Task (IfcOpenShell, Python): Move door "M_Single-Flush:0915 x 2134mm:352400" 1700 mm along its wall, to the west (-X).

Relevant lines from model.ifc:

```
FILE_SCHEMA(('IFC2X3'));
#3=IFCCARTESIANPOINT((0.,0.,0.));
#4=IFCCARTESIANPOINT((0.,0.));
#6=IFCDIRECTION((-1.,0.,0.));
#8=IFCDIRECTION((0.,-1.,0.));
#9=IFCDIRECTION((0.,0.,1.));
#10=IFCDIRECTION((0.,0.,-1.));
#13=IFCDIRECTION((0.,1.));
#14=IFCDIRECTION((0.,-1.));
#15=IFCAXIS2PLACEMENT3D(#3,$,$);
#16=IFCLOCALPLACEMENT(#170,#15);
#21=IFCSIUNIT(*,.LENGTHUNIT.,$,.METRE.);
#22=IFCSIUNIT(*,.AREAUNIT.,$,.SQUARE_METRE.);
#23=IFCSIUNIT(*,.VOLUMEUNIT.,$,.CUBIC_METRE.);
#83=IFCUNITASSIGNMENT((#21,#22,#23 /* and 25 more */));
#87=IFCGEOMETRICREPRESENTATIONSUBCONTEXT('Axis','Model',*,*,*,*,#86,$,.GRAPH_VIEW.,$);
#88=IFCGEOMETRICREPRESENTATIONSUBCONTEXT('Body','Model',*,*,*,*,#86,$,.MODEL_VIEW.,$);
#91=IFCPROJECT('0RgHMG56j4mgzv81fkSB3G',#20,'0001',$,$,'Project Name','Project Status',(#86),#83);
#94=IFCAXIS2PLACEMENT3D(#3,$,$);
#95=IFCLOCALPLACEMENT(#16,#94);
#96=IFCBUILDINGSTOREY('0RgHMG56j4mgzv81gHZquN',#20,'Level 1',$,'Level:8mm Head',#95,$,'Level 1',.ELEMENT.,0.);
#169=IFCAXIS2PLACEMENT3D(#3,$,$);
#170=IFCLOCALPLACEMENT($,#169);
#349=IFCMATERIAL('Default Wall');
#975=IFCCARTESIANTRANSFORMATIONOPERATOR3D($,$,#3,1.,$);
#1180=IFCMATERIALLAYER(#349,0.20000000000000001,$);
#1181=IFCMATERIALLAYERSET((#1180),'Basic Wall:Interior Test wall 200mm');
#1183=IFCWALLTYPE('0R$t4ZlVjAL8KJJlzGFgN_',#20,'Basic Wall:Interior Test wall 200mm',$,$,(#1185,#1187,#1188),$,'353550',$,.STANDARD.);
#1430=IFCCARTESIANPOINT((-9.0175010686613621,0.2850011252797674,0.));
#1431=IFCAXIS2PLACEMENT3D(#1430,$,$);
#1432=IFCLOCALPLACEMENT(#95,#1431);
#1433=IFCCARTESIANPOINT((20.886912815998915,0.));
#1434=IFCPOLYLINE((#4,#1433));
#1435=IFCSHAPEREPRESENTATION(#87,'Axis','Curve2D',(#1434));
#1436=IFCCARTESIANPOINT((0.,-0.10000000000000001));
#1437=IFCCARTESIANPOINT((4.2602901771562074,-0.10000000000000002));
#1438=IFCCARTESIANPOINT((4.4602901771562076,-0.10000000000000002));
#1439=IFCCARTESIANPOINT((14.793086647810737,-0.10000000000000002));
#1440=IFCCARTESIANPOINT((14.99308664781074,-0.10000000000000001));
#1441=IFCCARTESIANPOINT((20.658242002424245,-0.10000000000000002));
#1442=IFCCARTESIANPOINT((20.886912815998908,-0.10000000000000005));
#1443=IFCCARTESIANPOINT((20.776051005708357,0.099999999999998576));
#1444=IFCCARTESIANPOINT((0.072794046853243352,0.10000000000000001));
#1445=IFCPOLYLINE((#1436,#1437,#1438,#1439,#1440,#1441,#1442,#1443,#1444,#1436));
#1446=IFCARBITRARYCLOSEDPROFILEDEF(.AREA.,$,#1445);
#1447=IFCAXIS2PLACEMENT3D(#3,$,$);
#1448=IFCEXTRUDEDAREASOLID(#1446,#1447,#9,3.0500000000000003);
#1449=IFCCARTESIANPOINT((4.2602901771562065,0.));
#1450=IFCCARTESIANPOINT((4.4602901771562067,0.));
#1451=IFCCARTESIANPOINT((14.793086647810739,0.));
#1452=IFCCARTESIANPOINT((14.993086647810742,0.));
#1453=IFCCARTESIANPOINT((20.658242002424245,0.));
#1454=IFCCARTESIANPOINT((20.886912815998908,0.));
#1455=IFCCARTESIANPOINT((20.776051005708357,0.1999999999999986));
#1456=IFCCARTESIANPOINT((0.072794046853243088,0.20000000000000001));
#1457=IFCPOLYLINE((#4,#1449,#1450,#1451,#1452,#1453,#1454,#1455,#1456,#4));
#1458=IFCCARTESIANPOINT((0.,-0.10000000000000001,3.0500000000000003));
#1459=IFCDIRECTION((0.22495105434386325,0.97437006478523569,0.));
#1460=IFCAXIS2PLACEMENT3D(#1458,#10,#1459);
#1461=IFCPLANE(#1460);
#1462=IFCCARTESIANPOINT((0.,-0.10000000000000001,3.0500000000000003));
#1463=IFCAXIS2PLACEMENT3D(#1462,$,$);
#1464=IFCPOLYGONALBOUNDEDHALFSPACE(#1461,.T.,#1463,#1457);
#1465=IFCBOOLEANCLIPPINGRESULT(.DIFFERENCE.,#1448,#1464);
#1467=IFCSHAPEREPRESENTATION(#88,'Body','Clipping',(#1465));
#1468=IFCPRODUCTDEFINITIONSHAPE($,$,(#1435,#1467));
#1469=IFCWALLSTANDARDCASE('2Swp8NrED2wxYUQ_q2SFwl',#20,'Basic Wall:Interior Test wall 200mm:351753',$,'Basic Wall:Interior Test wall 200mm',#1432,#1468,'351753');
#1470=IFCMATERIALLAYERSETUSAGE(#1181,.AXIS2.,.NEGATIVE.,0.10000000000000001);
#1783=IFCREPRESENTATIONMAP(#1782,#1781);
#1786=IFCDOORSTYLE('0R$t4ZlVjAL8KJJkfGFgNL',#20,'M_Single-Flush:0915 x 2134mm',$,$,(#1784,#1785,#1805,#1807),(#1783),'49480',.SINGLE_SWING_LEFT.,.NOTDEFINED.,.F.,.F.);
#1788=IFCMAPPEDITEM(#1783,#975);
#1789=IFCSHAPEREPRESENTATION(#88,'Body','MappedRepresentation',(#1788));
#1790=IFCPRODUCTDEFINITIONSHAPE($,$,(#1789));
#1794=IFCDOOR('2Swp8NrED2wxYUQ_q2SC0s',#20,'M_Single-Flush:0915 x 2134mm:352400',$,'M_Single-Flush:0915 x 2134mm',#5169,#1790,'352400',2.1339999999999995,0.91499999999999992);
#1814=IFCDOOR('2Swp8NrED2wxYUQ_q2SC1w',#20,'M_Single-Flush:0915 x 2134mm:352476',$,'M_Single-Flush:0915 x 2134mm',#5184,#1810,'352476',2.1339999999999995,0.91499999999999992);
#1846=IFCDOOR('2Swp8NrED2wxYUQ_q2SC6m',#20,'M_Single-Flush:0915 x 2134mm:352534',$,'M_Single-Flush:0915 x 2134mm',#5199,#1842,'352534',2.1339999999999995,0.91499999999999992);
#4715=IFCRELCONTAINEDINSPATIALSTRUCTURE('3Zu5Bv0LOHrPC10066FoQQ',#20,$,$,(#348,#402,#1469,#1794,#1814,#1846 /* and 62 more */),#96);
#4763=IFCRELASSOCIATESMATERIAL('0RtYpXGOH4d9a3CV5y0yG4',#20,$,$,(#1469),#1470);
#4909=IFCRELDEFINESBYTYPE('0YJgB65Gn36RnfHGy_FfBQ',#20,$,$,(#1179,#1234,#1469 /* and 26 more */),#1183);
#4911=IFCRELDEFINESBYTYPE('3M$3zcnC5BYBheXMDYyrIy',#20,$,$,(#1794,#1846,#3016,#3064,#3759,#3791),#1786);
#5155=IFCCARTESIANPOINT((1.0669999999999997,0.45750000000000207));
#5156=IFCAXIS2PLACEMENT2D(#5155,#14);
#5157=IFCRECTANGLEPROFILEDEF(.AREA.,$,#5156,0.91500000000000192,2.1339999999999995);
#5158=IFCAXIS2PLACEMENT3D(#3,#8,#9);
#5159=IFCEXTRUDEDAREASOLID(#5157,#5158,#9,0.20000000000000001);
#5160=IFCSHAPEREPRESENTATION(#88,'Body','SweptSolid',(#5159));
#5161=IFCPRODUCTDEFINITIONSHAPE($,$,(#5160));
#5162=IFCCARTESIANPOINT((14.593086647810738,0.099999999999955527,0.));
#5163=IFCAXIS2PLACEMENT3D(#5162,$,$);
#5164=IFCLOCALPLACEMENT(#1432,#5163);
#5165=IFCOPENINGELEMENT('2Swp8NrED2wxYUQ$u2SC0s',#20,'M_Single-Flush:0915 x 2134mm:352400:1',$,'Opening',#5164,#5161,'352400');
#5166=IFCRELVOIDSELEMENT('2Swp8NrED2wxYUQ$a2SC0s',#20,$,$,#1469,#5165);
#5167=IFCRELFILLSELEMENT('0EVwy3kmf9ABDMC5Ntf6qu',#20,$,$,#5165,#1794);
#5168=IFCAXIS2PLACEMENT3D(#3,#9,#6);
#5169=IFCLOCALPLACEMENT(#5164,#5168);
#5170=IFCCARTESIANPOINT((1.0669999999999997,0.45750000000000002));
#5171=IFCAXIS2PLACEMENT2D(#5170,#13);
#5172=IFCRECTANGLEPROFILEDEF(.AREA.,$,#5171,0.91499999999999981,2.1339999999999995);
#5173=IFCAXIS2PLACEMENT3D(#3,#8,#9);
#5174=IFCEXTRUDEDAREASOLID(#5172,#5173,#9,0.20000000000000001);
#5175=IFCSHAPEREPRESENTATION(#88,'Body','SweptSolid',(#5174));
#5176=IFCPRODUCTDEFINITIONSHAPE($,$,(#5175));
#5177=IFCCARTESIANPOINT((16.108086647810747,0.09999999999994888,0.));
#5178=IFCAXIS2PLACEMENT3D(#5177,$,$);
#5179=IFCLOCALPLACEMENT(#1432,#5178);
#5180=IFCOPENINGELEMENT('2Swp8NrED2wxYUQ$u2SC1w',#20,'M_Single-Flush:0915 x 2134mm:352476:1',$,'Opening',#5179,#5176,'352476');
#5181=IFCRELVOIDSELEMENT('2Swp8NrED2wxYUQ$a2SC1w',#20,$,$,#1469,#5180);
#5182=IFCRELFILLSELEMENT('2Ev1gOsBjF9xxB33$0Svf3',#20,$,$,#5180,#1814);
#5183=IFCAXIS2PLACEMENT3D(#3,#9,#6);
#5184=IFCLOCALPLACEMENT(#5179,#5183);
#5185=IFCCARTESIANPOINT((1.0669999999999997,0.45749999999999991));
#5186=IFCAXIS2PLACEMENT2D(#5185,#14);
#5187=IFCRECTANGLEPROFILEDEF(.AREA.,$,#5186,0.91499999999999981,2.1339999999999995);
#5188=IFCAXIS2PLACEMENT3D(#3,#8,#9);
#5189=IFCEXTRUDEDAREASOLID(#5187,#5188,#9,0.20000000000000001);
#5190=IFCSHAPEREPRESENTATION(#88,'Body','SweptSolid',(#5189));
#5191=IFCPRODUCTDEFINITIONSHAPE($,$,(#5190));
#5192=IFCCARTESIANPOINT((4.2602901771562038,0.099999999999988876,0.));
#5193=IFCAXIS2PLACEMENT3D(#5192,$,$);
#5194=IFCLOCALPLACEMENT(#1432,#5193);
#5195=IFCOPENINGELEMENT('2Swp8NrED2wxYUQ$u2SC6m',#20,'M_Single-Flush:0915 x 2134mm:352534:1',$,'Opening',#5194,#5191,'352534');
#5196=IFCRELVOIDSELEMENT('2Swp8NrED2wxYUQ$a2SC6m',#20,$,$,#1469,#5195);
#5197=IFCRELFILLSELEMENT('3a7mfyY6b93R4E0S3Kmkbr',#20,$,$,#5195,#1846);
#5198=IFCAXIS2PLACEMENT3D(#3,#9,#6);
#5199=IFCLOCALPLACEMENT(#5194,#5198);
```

```python
import ifcopenshell
import ifcopenshell.api.geometry
import ifcopenshell.util.placement
import ifcopenshell.util.unit

model = ifcopenshell.open("model.ifc")
unit_scale = ifcopenshell.util.unit.calculate_unit_scale(model)

door = model.by_guid("2Swp8NrED2wxYUQ_q2SC0s")
opening = door.FillsVoids[0].RelatingOpeningElement
wall = opening.VoidsElements[0].RelatingBuildingElement

wall_matrix = ifcopenshell.util.placement.get_local_placement(wall.ObjectPlacement)
shift = wall_matrix[:3, 0] * -1.7 / unit_scale
before = ifcopenshell.util.placement.get_local_placement(door.ObjectPlacement)[:3, 3].copy()

# The door is placed relative to its opening, so it follows when the opening moves.
matrix = ifcopenshell.util.placement.get_local_placement(opening.ObjectPlacement)
matrix[:3, 3] += shift
ifcopenshell.api.geometry.edit_object_placement(
    model, product=opening, matrix=matrix, is_si=False, should_transform_children=True
)

after = ifcopenshell.util.placement.get_local_placement(door.ObjectPlacement)[:3, 3]
print("door moved by", (after - before).round(3) + 0.0)

model.write("model_updated.ifc")
```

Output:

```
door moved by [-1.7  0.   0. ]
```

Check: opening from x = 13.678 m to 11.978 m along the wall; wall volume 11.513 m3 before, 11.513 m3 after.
